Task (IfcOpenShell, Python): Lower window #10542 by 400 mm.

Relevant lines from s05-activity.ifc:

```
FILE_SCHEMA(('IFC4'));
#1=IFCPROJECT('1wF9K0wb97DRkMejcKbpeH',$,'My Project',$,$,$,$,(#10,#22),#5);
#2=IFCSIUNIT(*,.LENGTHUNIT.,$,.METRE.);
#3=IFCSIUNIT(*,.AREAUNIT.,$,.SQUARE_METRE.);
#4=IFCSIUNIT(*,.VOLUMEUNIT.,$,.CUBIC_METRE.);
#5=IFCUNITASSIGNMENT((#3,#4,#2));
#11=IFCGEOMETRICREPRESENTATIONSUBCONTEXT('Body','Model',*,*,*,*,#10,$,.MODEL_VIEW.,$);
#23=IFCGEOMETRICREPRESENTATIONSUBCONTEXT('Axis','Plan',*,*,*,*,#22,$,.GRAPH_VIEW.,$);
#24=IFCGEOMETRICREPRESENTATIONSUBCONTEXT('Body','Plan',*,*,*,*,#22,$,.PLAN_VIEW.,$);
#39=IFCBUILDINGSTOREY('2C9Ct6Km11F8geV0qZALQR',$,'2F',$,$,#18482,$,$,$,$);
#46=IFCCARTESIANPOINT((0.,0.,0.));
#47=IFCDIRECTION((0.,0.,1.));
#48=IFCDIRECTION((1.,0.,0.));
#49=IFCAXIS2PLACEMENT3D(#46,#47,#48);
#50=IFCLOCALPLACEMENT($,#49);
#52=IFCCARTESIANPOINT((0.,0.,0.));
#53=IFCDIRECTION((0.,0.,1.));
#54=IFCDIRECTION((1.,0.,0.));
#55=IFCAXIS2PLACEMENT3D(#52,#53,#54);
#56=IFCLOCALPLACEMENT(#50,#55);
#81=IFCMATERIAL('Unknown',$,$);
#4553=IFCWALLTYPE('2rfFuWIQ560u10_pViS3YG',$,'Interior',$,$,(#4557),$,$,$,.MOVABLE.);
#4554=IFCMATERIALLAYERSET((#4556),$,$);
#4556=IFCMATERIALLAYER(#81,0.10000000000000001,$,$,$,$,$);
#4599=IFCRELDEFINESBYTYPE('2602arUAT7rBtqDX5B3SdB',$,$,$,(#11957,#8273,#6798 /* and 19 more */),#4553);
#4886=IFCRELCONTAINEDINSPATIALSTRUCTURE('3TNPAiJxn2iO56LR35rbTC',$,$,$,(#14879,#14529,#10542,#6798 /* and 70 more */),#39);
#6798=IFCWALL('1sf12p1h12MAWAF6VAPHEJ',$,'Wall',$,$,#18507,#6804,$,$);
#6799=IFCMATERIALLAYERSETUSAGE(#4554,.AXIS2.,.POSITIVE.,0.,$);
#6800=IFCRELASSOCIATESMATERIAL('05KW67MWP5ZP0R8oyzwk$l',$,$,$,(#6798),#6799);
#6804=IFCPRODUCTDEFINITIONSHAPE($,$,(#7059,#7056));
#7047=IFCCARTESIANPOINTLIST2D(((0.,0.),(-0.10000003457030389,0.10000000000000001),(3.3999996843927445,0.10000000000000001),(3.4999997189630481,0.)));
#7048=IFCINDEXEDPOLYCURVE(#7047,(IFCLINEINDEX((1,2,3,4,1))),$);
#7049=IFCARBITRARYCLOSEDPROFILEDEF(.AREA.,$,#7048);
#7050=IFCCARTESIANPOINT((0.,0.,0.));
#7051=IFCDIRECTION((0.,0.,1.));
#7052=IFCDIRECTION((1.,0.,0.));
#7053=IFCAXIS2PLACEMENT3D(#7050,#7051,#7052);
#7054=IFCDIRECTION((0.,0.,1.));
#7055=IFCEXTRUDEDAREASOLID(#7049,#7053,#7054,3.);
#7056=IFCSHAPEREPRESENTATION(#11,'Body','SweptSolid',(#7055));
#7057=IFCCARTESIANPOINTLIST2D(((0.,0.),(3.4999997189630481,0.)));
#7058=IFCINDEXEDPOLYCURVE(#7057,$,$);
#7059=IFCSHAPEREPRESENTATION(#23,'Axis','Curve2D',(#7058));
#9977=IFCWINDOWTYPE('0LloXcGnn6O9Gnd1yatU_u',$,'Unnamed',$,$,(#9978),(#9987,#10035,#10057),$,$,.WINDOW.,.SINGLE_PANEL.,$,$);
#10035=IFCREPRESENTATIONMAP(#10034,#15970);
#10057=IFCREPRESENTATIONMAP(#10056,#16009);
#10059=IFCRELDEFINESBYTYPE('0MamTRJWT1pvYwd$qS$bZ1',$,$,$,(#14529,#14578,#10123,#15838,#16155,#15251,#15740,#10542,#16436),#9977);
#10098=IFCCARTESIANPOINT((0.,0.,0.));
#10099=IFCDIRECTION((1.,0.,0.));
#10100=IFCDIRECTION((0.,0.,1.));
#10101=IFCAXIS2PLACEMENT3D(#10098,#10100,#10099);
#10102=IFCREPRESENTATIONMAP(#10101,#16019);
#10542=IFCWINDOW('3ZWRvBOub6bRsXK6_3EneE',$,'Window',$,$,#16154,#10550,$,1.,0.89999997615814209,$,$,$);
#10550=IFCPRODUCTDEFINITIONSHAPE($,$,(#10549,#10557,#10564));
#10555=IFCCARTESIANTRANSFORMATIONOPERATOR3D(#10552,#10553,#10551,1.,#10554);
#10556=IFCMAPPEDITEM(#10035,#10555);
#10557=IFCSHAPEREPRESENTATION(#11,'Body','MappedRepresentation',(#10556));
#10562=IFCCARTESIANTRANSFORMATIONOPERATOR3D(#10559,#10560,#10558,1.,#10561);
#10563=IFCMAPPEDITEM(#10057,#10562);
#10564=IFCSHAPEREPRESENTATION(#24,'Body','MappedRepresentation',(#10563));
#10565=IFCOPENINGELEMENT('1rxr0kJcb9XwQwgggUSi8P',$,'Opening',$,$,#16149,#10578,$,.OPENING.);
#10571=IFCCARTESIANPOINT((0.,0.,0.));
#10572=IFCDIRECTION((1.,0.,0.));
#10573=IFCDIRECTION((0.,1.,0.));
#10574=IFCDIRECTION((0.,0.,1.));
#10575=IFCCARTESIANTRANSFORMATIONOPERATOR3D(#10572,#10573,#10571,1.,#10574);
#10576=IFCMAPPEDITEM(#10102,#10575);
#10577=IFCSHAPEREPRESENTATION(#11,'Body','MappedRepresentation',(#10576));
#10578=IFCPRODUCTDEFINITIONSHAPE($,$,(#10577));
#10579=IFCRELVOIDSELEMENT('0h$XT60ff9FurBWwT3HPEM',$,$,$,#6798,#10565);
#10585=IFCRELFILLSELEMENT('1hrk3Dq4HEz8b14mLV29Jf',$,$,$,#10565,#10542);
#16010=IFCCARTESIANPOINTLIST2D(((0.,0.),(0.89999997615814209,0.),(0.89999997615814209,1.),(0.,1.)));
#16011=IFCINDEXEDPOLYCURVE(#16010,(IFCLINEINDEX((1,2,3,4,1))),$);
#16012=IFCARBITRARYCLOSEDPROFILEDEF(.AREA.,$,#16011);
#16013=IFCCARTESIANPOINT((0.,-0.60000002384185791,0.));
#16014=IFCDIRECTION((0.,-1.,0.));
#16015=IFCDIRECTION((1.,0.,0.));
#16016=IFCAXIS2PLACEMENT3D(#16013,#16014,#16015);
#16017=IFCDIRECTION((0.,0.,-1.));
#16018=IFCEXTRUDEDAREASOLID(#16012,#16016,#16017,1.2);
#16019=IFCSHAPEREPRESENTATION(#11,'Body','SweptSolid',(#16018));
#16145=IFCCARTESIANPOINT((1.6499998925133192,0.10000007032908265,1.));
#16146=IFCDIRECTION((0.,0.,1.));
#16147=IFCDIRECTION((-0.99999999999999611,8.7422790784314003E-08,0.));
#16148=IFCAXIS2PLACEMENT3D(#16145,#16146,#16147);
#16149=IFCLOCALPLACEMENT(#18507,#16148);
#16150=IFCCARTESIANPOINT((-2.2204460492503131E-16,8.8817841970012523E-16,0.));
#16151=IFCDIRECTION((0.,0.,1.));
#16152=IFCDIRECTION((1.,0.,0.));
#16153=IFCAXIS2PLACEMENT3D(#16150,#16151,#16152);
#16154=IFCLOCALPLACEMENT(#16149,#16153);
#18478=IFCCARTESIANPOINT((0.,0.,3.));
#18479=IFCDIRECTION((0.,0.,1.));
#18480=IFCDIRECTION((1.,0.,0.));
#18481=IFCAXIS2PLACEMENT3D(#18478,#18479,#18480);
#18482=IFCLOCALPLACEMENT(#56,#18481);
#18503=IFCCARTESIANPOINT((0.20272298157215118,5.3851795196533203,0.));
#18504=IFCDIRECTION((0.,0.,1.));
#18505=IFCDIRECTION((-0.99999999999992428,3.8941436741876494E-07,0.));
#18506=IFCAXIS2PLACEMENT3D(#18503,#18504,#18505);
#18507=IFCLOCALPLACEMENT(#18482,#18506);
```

```python
import numpy as np
import ifcopenshell
import ifcopenshell.api.geometry
import ifcopenshell.util.placement
import ifcopenshell.util.unit

model = ifcopenshell.open("s05-activity.ifc")
unit_scale = ifcopenshell.util.unit.calculate_unit_scale(model)

window = model.by_guid("3ZWRvBOub6bRsXK6_3EneE")
opening = window.FillsVoids[0].RelatingOpeningElement
dz = -0.4 / unit_scale

shift = np.array([0.0, 0.0, dz])
# The window is placed relative to its opening, so it follows when the opening moves.
matrix = ifcopenshell.util.placement.get_local_placement(opening.ObjectPlacement)
matrix[:3, 3] += shift
ifcopenshell.api.geometry.edit_object_placement(
    model, product=opening, matrix=matrix, is_si=False, should_transform_children=True
)

print(f"moved by {dz * unit_scale:+.3f} m")

model.write("s05-activity_edited.ifc")
```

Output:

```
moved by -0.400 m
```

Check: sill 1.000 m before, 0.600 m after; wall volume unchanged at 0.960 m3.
